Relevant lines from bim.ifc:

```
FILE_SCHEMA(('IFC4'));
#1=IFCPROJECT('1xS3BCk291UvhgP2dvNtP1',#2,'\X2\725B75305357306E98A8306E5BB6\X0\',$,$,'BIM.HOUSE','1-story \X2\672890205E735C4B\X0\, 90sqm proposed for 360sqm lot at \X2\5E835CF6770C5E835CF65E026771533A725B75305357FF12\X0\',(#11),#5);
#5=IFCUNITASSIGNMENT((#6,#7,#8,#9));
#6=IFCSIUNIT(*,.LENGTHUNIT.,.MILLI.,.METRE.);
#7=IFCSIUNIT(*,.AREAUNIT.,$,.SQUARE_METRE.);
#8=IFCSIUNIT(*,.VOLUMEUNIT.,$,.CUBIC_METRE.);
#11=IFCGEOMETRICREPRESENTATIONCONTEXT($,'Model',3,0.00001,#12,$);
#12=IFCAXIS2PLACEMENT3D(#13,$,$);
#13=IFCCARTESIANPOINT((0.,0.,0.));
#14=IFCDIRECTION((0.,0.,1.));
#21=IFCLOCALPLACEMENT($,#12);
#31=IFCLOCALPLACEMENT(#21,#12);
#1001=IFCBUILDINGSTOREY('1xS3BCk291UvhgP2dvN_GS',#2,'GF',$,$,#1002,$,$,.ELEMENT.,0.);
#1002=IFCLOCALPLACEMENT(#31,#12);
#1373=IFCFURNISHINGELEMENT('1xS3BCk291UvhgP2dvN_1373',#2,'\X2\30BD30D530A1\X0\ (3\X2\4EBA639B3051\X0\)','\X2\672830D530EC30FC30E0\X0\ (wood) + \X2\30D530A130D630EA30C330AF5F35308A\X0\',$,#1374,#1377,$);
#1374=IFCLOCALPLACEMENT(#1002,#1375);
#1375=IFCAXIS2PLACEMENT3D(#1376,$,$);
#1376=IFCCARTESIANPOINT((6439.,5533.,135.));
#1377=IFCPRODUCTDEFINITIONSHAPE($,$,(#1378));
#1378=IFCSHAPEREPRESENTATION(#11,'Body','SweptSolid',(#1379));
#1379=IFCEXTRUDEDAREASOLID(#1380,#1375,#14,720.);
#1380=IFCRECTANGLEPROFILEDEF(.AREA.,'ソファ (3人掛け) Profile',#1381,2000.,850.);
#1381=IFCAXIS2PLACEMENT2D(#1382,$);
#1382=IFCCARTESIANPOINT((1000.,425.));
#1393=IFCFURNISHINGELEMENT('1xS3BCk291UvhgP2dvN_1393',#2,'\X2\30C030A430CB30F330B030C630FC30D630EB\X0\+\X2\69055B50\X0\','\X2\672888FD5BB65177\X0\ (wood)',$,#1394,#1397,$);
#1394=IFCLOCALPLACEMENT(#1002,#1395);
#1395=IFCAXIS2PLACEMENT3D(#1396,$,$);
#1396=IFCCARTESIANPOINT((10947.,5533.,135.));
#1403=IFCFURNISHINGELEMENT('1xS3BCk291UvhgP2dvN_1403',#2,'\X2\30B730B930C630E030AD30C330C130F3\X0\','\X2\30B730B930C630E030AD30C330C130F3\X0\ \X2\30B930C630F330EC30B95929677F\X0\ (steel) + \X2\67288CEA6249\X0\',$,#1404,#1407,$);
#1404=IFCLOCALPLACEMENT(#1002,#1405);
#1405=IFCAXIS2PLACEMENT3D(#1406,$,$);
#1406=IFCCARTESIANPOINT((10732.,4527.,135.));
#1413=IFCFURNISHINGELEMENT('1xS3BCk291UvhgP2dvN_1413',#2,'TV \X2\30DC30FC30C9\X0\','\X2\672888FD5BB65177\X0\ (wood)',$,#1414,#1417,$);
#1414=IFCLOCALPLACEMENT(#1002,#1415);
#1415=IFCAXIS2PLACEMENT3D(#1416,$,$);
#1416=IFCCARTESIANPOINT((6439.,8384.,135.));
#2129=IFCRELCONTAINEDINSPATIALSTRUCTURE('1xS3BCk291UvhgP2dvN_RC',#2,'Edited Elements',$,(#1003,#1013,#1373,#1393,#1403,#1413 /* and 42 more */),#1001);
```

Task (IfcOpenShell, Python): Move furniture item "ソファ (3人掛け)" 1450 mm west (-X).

```python
import ifcopenshell
import ifcopenshell.api.geometry
import ifcopenshell.util.placement

model = ifcopenshell.open("bim.ifc")

item = model.by_guid("1xS3BCk291UvhgP2dvN_1373")
matrix = ifcopenshell.util.placement.get_local_placement(item.ObjectPlacement)
matrix[0, 3] -= 1450.0
ifcopenshell.api.geometry.edit_object_placement(model, product=item, matrix=matrix, is_si=False)

print(ifcopenshell.util.placement.get_local_placement(item.ObjectPlacement).round(3) + 0.0)

model.write("bim_v2.ifc")
```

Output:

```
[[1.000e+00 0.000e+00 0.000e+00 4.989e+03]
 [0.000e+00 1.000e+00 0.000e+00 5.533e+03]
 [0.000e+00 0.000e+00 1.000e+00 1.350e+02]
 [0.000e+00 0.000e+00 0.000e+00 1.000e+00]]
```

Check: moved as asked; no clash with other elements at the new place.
